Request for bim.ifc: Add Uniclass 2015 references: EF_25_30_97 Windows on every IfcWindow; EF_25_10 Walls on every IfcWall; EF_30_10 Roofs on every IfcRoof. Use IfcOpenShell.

First a look at what the model holds.

```python
import ifcopenshell

model = ifcopenshell.open("bim.ifc")
print(model.schema)
print("classifications:", [c.Name for c in model.by_type("IfcClassification")])
for ifc_class in ("IfcDoor", "IfcRoof", "IfcStair", "IfcWall", "IfcWindow"):
    print(ifc_class, len(model.by_type(ifc_class)))
```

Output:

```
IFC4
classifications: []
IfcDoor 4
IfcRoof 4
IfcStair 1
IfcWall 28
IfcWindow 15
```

```python
import ifcopenshell
import ifcopenshell.api.classification

model = ifcopenshell.open("bim.ifc")

system = ifcopenshell.api.classification.add_classification(model, classification="Uniclass 2015")

codes = {
    "IfcWindow": ("EF_25_30_97", "Windows"),
    "IfcWall": ("EF_25_10", "Walls"),
    "IfcRoof": ("EF_30_10", "Roofs"),
}
for ifc_class, (code, name) in codes.items():
    products = model.by_type(ifc_class)
    ifcopenshell.api.classification.add_reference(
        model, products=products, classification=system, identification=code, name=name
    )
    print(code, len(products))

model.write("bim_rev.ifc")
```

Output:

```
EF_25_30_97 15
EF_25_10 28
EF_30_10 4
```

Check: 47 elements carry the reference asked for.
